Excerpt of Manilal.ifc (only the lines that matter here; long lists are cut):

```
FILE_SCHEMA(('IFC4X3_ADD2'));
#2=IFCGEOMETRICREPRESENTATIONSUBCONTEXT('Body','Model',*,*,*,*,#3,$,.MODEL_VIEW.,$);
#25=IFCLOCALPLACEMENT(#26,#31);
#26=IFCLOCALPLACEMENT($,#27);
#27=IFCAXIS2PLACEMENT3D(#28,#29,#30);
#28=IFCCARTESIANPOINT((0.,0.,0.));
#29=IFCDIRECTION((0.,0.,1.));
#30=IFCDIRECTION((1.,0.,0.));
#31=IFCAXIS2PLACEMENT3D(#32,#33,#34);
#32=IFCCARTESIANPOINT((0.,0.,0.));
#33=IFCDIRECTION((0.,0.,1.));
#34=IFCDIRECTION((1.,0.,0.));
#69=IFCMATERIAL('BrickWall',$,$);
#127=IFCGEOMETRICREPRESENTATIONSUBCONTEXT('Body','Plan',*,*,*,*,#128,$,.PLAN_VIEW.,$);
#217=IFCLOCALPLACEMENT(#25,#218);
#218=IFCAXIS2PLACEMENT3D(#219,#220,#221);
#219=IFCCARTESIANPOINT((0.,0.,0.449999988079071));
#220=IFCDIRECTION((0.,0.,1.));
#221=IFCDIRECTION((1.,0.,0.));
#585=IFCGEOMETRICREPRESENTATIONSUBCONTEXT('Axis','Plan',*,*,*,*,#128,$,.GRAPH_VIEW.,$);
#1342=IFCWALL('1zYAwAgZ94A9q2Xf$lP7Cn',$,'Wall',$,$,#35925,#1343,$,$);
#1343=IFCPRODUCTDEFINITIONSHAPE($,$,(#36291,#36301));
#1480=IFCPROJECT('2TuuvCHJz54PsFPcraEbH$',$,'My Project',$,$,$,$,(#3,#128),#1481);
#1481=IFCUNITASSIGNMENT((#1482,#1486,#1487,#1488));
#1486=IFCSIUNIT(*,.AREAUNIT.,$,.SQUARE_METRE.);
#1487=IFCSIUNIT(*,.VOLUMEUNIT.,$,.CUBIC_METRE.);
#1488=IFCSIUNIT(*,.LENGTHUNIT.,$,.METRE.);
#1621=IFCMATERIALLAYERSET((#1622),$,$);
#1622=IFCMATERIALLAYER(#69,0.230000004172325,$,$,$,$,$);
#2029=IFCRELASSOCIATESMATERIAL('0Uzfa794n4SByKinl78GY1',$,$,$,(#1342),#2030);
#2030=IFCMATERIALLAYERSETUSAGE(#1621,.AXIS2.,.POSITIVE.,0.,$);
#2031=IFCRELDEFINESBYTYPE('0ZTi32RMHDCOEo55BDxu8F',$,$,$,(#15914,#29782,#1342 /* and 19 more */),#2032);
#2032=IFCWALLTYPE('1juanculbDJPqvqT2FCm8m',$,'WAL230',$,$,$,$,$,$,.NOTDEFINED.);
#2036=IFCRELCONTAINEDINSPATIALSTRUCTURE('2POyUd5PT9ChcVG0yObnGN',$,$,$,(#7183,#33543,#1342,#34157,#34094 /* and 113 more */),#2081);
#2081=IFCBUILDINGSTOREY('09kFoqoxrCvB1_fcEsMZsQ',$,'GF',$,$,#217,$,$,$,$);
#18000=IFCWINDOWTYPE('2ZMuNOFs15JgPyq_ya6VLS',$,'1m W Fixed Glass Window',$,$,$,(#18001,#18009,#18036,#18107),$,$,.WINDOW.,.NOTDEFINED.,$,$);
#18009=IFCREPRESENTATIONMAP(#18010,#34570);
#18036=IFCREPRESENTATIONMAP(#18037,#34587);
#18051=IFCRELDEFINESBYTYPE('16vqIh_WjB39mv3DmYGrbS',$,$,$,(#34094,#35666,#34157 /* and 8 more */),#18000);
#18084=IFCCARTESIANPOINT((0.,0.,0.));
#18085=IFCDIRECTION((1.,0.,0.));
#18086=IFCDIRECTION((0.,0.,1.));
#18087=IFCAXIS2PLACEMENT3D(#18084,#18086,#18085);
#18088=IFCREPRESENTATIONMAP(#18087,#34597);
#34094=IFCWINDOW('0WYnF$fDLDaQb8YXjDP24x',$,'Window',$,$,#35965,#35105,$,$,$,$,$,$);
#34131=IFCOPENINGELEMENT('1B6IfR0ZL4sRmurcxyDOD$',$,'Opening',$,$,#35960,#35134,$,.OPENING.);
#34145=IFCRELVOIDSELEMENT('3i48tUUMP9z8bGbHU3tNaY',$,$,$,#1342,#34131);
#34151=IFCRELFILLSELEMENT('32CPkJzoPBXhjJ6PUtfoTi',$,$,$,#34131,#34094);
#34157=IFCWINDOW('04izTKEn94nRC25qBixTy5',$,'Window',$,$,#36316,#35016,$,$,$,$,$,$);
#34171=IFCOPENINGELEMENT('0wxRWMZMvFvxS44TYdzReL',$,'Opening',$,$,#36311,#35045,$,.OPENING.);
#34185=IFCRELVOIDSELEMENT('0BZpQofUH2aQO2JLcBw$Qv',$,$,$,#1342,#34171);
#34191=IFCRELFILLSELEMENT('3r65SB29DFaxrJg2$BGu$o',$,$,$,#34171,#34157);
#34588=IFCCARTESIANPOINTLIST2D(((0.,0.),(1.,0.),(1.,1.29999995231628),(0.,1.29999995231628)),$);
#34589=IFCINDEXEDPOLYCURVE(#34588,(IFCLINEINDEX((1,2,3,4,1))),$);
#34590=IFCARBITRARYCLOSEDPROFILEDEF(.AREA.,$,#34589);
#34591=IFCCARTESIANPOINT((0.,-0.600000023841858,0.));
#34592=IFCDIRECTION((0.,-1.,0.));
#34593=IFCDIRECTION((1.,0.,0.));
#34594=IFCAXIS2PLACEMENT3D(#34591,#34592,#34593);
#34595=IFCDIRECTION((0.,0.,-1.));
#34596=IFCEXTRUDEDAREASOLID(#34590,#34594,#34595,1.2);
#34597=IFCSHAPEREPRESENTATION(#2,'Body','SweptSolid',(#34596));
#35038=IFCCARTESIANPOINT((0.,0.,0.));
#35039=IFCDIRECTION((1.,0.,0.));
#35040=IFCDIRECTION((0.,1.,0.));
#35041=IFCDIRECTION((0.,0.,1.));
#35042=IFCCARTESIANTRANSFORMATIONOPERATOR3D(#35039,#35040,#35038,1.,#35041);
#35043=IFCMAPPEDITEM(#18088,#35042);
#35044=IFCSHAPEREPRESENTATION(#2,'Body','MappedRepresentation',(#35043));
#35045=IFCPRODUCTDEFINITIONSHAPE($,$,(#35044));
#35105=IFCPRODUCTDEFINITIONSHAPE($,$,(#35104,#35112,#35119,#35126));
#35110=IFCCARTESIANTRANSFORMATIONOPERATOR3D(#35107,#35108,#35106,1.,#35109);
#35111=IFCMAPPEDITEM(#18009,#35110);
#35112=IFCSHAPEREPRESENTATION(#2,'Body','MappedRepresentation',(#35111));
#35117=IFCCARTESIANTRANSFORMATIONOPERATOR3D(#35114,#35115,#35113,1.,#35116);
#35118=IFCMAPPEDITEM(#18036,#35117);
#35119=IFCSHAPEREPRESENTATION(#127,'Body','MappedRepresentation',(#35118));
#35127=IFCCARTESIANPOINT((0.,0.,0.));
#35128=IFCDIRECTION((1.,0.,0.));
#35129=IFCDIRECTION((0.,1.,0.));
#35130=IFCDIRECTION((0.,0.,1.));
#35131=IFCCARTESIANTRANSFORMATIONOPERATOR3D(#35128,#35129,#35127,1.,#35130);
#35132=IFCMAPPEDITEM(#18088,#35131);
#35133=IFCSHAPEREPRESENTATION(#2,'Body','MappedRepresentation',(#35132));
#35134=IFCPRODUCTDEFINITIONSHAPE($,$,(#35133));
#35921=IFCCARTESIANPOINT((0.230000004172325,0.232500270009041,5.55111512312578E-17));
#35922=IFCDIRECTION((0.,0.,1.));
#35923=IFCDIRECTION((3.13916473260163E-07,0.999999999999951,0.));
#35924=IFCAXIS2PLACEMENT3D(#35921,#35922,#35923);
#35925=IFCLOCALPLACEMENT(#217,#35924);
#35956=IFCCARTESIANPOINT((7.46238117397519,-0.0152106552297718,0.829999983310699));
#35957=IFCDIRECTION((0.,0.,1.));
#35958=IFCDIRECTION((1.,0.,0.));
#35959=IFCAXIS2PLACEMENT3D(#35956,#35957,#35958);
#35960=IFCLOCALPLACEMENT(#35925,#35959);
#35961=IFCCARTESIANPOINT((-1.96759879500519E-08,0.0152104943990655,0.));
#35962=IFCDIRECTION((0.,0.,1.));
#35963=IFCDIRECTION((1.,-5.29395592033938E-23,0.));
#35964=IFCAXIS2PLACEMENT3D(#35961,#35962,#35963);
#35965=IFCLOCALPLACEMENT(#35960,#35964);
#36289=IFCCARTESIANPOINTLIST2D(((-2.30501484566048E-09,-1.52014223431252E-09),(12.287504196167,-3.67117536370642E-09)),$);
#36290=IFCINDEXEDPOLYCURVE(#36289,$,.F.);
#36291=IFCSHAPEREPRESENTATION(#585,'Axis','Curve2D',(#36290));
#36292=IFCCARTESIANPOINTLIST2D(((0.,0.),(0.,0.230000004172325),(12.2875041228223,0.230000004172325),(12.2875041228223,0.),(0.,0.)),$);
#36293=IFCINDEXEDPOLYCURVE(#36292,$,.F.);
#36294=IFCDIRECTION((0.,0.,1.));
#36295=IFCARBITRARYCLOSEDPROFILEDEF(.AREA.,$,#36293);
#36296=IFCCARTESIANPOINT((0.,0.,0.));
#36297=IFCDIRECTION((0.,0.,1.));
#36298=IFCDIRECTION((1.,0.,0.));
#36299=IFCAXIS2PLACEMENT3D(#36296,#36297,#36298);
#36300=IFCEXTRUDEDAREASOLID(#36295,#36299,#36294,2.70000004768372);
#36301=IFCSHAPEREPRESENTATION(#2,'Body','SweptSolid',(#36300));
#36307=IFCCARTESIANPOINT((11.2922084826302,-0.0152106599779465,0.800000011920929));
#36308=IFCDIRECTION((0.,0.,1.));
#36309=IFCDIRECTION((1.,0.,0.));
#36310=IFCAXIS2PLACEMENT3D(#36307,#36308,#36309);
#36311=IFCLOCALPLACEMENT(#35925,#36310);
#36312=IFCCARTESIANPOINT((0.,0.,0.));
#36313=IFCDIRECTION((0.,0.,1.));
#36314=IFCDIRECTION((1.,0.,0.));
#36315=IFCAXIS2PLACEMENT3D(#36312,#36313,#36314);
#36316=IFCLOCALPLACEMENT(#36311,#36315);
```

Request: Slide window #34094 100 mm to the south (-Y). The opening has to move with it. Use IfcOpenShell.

```python
import ifcopenshell
import ifcopenshell.api.geometry
import ifcopenshell.util.placement

model = ifcopenshell.open("Manilal.ifc")

window = model.by_guid("0WYnF$fDLDaQb8YXjDP24x")
opening = window.FillsVoids[0].RelatingOpeningElement
wall = opening.VoidsElements[0].RelatingBuildingElement

wall_matrix = ifcopenshell.util.placement.get_local_placement(wall.ObjectPlacement)
shift = wall_matrix[:3, 0] * -0.1
before = ifcopenshell.util.placement.get_local_placement(window.ObjectPlacement)[:3, 3].copy()

# The window is placed relative to its opening, so it follows when the opening moves.
matrix = ifcopenshell.util.placement.get_local_placement(opening.ObjectPlacement)
matrix[:3, 3] += shift
ifcopenshell.api.geometry.edit_object_placement(
    model, product=opening, matrix=matrix, is_si=False, should_transform_children=True
)

after = ifcopenshell.util.placement.get_local_placement(window.ObjectPlacement)[:3, 3]
print("window moved by", (after - before).round(3) + 0.0)

model.write("Manilal_rev.ifc")
```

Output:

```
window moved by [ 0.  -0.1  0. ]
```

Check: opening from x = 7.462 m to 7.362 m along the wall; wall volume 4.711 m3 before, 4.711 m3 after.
